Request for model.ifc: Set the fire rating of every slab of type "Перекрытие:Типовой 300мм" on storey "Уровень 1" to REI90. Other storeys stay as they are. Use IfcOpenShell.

First a look at what the model holds.

```python
import ifcopenshell
import ifcopenshell.util.element

model = ifcopenshell.open("model.ifc")
print(model.schema)
storey = next(s for s in model.by_type("IfcBuildingStorey") if s.Name == "Уровень 1")
slabs = [e for e in ifcopenshell.util.element.get_decomposition(storey) if e.is_a("IfcSlab")]
seen = {}
for e in slabs:
    element_type = ifcopenshell.util.element.get_type(e)
    key = (element_type.Name if element_type != e and element_type else None, ifcopenshell.util.element.get_pset(e, "Pset_SlabCommon", "FireRating"))
    seen[key] = seen.get(key, 0) + 1
for (name, value), count in sorted(seen.items(), key=str):
    print(count, "x", name, "|", value)
```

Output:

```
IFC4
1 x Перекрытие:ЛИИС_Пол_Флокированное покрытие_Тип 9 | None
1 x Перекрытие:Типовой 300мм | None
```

```python
import ifcopenshell
import ifcopenshell.api.pset
import ifcopenshell.util.element

model = ifcopenshell.open("model.ifc")

storey = next(s for s in model.by_type("IfcBuildingStorey") if s.Name == "Уровень 1")
slabs = [e for e in ifcopenshell.util.element.get_decomposition(storey) if e.is_a("IfcSlab")]

count = 0
for e in slabs:
    element_type = ifcopenshell.util.element.get_type(e)
    if element_type in (None, e) or element_type.Name != "Перекрытие:Типовой 300мм":
        continue
    # add_pset returns the element's existing set when there is one.
    pset = ifcopenshell.api.pset.add_pset(model, product=e, name="Pset_SlabCommon")
    ifcopenshell.api.pset.edit_pset(model, pset=pset, properties={"FireRating": "REI90"})
    count += 1

print(count, "slabs updated")

model.write("model_edited.ifc")
```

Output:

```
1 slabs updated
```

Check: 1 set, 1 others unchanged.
